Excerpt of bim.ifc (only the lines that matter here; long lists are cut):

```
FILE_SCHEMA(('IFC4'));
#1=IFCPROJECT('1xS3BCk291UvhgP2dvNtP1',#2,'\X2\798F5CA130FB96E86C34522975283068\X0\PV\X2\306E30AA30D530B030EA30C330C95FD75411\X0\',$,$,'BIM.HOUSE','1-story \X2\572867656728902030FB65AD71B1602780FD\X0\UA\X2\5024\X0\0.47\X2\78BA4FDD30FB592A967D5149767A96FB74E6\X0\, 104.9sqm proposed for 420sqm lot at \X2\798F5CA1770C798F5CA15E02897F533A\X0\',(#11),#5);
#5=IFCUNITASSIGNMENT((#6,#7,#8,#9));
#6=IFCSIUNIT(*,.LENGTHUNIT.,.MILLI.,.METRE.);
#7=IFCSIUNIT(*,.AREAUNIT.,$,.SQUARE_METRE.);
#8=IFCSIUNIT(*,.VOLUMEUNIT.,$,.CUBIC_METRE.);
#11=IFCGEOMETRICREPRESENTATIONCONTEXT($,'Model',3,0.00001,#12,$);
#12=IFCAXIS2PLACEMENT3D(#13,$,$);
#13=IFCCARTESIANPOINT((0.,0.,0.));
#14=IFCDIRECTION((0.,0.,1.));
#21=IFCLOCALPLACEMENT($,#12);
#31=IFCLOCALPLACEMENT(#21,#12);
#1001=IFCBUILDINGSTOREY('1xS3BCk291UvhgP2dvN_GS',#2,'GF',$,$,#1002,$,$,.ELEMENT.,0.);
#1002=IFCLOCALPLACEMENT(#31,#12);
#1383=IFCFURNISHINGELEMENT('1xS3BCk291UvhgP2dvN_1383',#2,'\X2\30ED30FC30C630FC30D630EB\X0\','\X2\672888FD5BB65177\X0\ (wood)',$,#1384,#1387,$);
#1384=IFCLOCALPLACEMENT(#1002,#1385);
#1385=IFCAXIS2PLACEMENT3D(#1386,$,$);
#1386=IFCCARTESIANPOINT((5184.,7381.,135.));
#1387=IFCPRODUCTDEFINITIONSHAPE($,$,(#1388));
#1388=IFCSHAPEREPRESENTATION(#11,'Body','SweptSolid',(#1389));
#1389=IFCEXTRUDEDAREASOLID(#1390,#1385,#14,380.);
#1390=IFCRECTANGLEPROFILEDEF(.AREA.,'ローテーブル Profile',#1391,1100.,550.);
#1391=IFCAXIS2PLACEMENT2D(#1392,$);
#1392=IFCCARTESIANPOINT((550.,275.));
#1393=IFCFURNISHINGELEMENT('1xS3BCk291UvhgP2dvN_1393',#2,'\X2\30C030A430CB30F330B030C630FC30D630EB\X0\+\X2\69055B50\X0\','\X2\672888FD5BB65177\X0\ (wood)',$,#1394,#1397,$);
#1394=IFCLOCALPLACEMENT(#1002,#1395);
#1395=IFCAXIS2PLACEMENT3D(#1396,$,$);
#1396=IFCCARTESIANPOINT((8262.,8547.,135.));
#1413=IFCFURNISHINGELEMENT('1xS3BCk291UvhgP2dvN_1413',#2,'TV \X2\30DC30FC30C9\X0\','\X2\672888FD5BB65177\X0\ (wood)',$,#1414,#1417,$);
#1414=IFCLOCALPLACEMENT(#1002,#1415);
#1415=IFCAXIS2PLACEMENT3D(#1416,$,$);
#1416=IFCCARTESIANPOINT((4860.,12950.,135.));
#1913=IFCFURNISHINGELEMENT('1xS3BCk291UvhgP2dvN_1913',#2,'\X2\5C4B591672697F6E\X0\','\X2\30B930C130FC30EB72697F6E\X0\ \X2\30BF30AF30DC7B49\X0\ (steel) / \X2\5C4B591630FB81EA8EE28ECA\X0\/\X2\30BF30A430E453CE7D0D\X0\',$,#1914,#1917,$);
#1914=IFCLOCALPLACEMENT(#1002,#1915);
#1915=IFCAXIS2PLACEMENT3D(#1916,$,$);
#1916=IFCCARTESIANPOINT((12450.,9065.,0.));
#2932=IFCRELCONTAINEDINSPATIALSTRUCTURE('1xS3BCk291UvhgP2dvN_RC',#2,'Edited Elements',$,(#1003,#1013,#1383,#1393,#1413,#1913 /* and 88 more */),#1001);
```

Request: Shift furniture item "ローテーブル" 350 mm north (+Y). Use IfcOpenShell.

```python
import ifcopenshell
import ifcopenshell.api.geometry
import ifcopenshell.util.placement
import ifcopenshell.util.unit

model = ifcopenshell.open("bim.ifc")
unit_scale = ifcopenshell.util.unit.calculate_unit_scale(model)

item = model.by_id(1383)
matrix = ifcopenshell.util.placement.get_local_placement(item.ObjectPlacement)
matrix[1, 3] += 0.35 / unit_scale
ifcopenshell.api.geometry.edit_object_placement(model, product=item, matrix=matrix, is_si=False)

print(ifcopenshell.util.placement.get_local_placement(item.ObjectPlacement).round(3) + 0.0)

model.write("bim_rev.ifc")
```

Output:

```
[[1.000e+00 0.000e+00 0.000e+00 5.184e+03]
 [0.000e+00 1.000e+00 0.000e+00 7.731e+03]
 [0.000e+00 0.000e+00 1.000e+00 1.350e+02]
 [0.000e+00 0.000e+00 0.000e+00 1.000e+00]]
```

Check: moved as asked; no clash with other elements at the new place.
